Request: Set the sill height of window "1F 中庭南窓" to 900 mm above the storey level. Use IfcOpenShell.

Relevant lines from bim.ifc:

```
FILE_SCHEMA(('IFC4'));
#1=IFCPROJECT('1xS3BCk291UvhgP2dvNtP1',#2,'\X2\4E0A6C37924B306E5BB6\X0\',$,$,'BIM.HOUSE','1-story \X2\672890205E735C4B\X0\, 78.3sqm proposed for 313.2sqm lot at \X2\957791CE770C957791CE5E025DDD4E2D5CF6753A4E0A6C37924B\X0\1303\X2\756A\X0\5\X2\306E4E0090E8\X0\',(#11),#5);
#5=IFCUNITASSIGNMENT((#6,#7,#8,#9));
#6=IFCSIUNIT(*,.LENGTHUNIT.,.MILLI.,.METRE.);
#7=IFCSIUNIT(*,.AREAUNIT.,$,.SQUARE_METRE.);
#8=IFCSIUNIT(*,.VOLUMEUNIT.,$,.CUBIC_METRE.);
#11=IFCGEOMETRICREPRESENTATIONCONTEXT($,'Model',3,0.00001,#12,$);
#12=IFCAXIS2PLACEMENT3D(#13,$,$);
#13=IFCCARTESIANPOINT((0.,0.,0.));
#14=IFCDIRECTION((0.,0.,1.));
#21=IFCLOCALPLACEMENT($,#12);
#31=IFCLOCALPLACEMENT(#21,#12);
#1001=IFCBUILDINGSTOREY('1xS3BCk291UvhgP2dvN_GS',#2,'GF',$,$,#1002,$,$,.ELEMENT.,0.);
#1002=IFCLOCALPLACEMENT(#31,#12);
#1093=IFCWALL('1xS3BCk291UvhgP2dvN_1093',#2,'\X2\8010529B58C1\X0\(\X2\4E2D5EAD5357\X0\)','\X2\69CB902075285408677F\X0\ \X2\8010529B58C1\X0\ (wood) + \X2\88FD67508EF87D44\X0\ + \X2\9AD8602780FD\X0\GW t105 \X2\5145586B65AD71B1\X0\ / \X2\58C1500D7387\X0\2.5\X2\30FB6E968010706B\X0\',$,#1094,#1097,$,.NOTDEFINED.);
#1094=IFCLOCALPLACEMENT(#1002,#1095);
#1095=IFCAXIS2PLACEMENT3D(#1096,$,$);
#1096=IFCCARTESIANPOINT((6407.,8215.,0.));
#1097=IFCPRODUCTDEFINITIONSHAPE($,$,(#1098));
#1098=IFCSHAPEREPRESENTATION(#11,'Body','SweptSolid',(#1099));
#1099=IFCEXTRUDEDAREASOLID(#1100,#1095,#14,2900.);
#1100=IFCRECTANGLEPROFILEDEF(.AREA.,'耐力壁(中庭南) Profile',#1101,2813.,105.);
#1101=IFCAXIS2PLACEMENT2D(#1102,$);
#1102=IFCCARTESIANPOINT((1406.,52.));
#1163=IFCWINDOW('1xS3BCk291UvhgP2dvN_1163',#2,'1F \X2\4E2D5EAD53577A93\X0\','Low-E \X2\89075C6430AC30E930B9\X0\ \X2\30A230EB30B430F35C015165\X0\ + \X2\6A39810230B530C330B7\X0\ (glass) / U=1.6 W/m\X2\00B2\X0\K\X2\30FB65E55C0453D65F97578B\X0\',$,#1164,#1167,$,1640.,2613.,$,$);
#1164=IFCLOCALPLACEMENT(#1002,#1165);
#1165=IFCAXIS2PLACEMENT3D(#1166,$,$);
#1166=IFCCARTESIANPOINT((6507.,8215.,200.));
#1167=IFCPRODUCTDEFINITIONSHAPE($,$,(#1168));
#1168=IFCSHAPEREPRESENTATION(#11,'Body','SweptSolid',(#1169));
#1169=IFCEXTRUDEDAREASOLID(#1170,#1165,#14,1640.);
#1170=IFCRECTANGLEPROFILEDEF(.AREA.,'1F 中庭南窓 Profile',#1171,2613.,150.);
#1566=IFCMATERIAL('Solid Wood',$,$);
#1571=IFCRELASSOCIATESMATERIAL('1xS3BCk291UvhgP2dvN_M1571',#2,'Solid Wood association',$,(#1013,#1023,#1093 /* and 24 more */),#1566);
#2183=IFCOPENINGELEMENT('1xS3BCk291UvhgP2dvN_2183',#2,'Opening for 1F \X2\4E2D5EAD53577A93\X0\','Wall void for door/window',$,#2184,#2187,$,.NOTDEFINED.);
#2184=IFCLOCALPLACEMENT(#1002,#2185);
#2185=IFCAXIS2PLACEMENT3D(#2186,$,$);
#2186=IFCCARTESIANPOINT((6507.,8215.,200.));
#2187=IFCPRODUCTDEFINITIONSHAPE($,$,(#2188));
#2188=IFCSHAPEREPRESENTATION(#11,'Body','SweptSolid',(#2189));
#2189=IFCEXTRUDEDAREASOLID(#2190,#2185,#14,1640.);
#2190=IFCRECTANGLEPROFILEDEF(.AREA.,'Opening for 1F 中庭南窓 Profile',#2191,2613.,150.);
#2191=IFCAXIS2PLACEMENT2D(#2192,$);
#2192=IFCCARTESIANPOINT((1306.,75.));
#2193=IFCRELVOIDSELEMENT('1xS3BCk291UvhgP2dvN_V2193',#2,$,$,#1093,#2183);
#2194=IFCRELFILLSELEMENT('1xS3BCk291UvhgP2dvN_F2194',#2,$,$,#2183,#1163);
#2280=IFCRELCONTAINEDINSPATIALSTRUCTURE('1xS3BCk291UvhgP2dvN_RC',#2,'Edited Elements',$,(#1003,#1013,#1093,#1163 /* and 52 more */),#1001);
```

```python
import numpy as np
import ifcopenshell
import ifcopenshell.api.geometry
import ifcopenshell.geom
import ifcopenshell.util.element
import ifcopenshell.util.placement
import ifcopenshell.util.shape
import ifcopenshell.util.unit

model = ifcopenshell.open("bim.ifc")
unit_scale = ifcopenshell.util.unit.calculate_unit_scale(model)

window = model.by_guid("1xS3BCk291UvhgP2dvN_1163")
opening = window.FillsVoids[0].RelatingOpeningElement
storey = ifcopenshell.util.element.get_container(window, ifc_class="IfcBuildingStorey")
level = ifcopenshell.util.placement.get_local_placement(storey.ObjectPlacement)[2, 3]

# The opening's origin need not be at the sill, so measure its lowest point.
shape = ifcopenshell.geom.create_shape(ifcopenshell.geom.settings(), opening)
bottom = ifcopenshell.util.shape.get_shape_bottom_elevation(shape, shape.geometry) / unit_scale
dz = level + 0.9 / unit_scale - bottom

shift = np.array([0.0, 0.0, dz])
# The window is not placed relative to its opening, so move both.
for product in (opening, window):
    matrix = ifcopenshell.util.placement.get_local_placement(product.ObjectPlacement)
    matrix[:3, 3] += shift
    ifcopenshell.api.geometry.edit_object_placement(model, product=product, matrix=matrix, is_si=False)

print(f"moved by {dz * unit_scale:+.3f} m")

model.write("bim_updated.ifc")
```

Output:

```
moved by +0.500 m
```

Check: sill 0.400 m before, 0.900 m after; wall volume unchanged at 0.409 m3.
